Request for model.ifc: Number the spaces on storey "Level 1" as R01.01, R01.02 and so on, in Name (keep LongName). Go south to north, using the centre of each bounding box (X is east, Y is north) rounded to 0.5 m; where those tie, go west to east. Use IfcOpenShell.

First a look at what the model holds.

```python
import ifcopenshell
import ifcopenshell.util.element
import ifcopenshell.util.placement

model = ifcopenshell.open("model.ifc")
print(model.schema)
storey = next(s for s in model.by_type("IfcBuildingStorey") if s.Name == "Level 1")
spaces = [e for e in ifcopenshell.util.element.get_decomposition(storey) if e.is_a("IfcSpace")]
for e in sorted(spaces, key=lambda e: e.id()):
    origin = ifcopenshell.util.placement.get_local_placement(e.ObjectPlacement)[:3, 3]
    print(e.id(), e.Name, e.LongName, origin.round(2) + 0.0, sep=" | ")
```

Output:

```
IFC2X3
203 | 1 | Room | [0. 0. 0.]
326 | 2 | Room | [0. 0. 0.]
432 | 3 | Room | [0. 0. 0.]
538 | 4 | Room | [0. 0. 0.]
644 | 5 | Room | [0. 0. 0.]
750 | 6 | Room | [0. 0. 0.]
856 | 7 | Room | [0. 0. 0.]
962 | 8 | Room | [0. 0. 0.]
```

```python
import ifcopenshell
import ifcopenshell.geom
import ifcopenshell.util.element
import ifcopenshell.util.shape

model = ifcopenshell.open("model.ifc")
settings = ifcopenshell.geom.settings()
settings.set("use-world-coords", True)


def centre(element):
    shape = ifcopenshell.geom.create_shape(settings, element)
    return ifcopenshell.util.shape.get_bbox_centroid(shape.geometry)


storey = next(s for s in model.by_type("IfcBuildingStorey") if s.Name == "Level 1")
spaces = [e for e in ifcopenshell.util.element.get_decomposition(storey) if e.is_a("IfcSpace")]

# Insertion points can sit at a corner or the storey origin, so sort by the geometry (in metres).
centres = {e: centre(e) for e in spaces}
spaces.sort(key=lambda e: (round(centres[e][1] / 0.5), centres[e][0]))

for i, e in enumerate(spaces, start=1):
    number = f"R01.{i:02d}"
    e.Name = number
    print(e.id(), number)

model.write("model_v2.ifc")
```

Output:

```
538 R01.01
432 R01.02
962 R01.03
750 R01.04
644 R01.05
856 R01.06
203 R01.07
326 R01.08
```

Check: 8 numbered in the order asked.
